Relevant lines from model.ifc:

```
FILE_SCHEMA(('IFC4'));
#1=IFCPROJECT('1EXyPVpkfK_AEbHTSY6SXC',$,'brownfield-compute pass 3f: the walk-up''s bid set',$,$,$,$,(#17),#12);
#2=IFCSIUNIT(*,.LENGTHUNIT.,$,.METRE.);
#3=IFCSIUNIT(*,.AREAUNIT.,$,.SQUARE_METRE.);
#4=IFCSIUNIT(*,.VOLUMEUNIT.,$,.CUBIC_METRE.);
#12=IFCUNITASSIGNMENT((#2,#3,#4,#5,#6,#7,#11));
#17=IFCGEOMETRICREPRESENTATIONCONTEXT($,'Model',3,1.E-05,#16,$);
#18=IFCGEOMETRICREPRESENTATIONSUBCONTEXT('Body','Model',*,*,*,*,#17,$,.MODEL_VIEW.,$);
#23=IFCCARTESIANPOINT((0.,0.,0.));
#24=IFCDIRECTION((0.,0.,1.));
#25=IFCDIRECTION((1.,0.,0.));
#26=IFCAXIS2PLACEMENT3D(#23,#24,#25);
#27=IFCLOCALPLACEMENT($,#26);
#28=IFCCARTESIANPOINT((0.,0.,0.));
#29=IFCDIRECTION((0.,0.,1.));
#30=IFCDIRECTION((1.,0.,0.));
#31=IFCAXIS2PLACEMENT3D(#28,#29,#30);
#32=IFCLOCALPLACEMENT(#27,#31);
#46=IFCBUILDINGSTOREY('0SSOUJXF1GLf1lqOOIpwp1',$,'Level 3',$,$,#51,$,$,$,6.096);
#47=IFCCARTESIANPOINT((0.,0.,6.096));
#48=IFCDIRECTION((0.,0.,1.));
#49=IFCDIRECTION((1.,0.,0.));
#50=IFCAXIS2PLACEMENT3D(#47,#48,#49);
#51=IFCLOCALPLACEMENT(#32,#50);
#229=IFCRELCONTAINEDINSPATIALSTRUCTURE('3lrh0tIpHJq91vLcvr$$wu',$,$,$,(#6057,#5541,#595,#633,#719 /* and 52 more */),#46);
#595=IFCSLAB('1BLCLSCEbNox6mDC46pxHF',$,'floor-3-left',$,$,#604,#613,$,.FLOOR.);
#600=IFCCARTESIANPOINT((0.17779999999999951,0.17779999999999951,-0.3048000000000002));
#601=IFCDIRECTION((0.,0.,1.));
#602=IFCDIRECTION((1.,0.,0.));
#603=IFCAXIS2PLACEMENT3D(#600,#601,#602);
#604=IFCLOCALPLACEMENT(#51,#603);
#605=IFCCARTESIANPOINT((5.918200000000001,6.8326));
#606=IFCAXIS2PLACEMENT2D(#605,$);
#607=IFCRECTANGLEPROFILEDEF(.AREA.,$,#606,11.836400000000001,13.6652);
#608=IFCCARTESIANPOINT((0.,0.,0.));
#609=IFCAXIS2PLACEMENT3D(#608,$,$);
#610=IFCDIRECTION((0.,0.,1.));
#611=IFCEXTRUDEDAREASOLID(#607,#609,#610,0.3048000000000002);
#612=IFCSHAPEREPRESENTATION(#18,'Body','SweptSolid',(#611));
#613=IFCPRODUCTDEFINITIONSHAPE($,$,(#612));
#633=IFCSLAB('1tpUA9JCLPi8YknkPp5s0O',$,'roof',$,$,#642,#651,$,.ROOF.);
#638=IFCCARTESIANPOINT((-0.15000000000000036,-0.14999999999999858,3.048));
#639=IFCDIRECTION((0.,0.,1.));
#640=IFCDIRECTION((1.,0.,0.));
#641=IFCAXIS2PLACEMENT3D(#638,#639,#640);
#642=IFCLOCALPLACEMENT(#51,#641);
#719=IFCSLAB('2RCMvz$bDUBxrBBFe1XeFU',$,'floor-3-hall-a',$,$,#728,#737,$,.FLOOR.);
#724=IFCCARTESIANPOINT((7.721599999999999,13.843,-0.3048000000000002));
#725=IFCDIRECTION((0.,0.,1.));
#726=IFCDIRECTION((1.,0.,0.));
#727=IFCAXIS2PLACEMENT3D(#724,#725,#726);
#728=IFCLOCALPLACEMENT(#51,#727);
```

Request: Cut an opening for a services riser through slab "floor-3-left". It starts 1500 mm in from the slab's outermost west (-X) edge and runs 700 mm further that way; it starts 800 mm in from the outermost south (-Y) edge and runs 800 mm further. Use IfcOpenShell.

```python
import numpy as np
import ifcopenshell
import ifcopenshell.api.feature
import ifcopenshell.api.geometry
import ifcopenshell.api.root
import ifcopenshell.geom
import ifcopenshell.util.placement
import ifcopenshell.util.representation
import ifcopenshell.util.shape
import ifcopenshell.util.unit

model = ifcopenshell.open("model.ifc")
unit_scale = ifcopenshell.util.unit.calculate_unit_scale(model)
settings = ifcopenshell.geom.settings()


def volume(element):
    """Net volume in cubic metres, openings subtracted."""
    shape = ifcopenshell.geom.create_shape(settings, element)
    return ifcopenshell.util.shape.get_volume(shape.geometry)


slab = model.by_guid("1BLCLSCEbNox6mDC46pxHF")
before = volume(slab)

# Extent in the slab's own axes, in metres. The edges named are its -X and -Y sides.
slab_shape = ifcopenshell.geom.create_shape(settings, slab)
vertices = ifcopenshell.util.shape.get_vertices(slab_shape.geometry)
x_min, y_min, bottom = vertices.min(axis=0)
top = vertices[:, 2].max()

opening = ifcopenshell.api.root.create_entity(model, ifc_class="IfcOpeningElement", name="Services riser opening", predefined_type="OPENING")
context = ifcopenshell.util.representation.get_context(model, "Model", "Body", "MODEL_VIEW")
width, depth = 0.7, 0.8
outline = [(0.0, 0.0), (width, 0.0), (width, depth), (0.0, depth), (0.0, 0.0)]
# Overshoot both faces by 50 mm so the cut is clean.
shape = ifcopenshell.api.geometry.add_slab_representation(
    model, context=context, depth=top - bottom + 0.1, polyline=outline
)
ifcopenshell.api.geometry.assign_representation(model, product=opening, representation=shape)

matrix = ifcopenshell.util.placement.get_local_placement(slab.ObjectPlacement)
matrix[:, 3] = matrix @ np.append(np.array([x_min + 1.5, y_min + 0.8, bottom - 0.05]) / unit_scale, 1.0)
ifcopenshell.api.geometry.edit_object_placement(model, product=opening, matrix=matrix, is_si=False)
ifcopenshell.api.feature.add_feature(model, feature=opening, element=slab)

after = volume(slab)

print(f"slab volume {before:.3f} -> {after:.3f} m3")

model.write("model_updated.ifc")
```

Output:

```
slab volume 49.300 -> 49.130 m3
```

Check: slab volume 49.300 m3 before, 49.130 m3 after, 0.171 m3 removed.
